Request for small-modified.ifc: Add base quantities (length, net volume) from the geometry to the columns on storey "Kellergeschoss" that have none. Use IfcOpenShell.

First a look at what the model holds.

```python
import ifcopenshell
import ifcopenshell.util.element
import ifcopenshell.util.unit

model = ifcopenshell.open("small-modified.ifc")
print(model.schema)
for unit_type in ("LENGTHUNIT", "AREAUNIT", "VOLUMEUNIT"):
    print(unit_type, ifcopenshell.util.unit.calculate_unit_scale(model, unit_type))
storey = next(s for s in model.by_type("IfcBuildingStorey") if s.Name == "Kellergeschoss")
columns = [e for e in ifcopenshell.util.element.get_decomposition(storey) if e.is_a("IfcColumn")]
for e in sorted(columns, key=lambda e: e.id()):
    print(e.id(), e.is_a(), e.Name, list(ifcopenshell.util.element.get_psets(e, qtos_only=True)), sep=" | ")
```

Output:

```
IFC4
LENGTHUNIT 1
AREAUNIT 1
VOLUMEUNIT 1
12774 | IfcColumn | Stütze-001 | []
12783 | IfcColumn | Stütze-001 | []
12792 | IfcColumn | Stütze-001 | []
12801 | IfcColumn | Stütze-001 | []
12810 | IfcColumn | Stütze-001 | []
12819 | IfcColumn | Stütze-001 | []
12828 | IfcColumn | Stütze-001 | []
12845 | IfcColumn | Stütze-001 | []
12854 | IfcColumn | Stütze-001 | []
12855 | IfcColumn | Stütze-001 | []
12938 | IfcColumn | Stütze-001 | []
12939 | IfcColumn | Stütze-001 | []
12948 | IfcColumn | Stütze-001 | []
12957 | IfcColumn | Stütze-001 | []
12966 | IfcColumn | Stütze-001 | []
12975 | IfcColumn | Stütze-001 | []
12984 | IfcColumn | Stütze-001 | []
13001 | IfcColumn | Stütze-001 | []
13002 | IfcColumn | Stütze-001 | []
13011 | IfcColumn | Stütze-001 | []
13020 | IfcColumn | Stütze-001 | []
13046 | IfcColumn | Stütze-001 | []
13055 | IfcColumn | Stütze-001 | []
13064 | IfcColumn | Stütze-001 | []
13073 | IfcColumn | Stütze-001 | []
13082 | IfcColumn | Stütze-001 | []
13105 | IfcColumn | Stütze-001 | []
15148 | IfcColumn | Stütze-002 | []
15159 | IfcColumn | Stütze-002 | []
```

```python
import ifcopenshell
import ifcopenshell.api.pset
import ifcopenshell.geom
import ifcopenshell.util.element
import ifcopenshell.util.shape
import ifcopenshell.util.unit

model = ifcopenshell.open("small-modified.ifc")
unit_scale = ifcopenshell.util.unit.calculate_unit_scale(model)
volume_scale = ifcopenshell.util.unit.calculate_unit_scale(model, "VOLUMEUNIT")
settings = ifcopenshell.geom.settings()

storey = next(s for s in model.by_type("IfcBuildingStorey") if s.Name == "Kellergeschoss")
columns = [e for e in ifcopenshell.util.element.get_decomposition(storey) if e.is_a("IfcColumn")]

for e in sorted(columns, key=lambda e: e.id()):
    if ifcopenshell.util.element.get_psets(e, qtos_only=True, should_inherit=False):
        continue
    # Geometry comes back in metres, in the element's own axes.
    shape = ifcopenshell.geom.create_shape(settings, e)
    values = {
        "Length": ifcopenshell.util.shape.get_z(shape.geometry) / unit_scale,
        "NetVolume": ifcopenshell.util.shape.get_volume(shape.geometry) / volume_scale,
    }
    qto = ifcopenshell.api.pset.add_qto(model, product=e, name="Qto_ColumnBaseQuantities")
    ifcopenshell.api.pset.edit_qto(model, qto=qto, properties=values)
    print(e.id(), {k: round(v, 3) for k, v in values.items()})

model.write("small-modified_edited.ifc")
```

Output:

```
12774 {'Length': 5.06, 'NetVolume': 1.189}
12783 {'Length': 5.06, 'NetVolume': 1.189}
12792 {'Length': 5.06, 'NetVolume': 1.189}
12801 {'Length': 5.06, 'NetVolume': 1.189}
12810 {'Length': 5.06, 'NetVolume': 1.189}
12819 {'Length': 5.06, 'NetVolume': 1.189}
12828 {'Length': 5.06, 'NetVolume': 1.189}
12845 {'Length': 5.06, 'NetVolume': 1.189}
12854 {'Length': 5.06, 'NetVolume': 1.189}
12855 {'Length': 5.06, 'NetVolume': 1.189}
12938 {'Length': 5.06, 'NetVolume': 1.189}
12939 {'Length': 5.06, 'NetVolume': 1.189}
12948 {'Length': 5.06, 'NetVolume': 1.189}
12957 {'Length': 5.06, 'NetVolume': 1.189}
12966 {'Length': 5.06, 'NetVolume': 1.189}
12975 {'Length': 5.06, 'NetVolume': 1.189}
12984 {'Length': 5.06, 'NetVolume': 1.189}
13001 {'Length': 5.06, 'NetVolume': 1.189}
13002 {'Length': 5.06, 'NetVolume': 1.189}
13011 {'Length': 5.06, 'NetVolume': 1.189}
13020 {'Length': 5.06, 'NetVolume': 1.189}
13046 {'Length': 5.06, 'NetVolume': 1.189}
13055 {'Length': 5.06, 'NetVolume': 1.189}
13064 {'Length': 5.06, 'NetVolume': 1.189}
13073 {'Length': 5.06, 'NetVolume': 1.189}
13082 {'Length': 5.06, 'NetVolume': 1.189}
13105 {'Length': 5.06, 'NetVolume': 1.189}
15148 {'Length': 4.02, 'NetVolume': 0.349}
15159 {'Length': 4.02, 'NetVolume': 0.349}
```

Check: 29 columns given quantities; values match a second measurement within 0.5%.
